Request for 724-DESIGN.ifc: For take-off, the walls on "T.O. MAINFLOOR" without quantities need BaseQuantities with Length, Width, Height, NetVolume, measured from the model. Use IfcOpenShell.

First a look at what the model holds.

```python
import ifcopenshell
import ifcopenshell.util.element
import ifcopenshell.util.unit

model = ifcopenshell.open("724-DESIGN.ifc")
print(model.schema)
for unit_type in ("LENGTHUNIT", "AREAUNIT", "VOLUMEUNIT"):
    print(unit_type, ifcopenshell.util.unit.calculate_unit_scale(model, unit_type))
storey = next(s for s in model.by_type("IfcBuildingStorey") if s.Name == "T.O. MAINFLOOR")
walls = [e for e in ifcopenshell.util.element.get_decomposition(storey) if e.is_a("IfcWall")]
for e in sorted(walls, key=lambda e: e.id()):
    print(e.id(), e.is_a(), e.Name, list(ifcopenshell.util.element.get_psets(e, qtos_only=True)), sep=" | ")
```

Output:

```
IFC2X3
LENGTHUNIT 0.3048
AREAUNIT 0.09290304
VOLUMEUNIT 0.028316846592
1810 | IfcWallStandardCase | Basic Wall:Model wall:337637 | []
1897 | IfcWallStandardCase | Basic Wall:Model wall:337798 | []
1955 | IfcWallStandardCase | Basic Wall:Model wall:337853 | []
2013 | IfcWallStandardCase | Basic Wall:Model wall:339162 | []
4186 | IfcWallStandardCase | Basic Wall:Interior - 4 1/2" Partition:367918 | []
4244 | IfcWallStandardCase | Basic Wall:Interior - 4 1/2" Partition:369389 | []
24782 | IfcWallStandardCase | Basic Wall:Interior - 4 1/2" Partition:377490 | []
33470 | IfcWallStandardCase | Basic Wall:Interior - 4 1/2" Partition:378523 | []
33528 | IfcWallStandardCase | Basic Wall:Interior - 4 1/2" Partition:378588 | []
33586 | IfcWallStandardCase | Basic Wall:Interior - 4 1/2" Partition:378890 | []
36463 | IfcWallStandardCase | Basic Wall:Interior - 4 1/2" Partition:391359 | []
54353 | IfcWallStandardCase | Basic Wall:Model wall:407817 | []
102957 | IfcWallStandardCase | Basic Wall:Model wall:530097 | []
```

```python
import ifcopenshell
import ifcopenshell.api.pset
import ifcopenshell.geom
import ifcopenshell.util.element
import ifcopenshell.util.shape
import ifcopenshell.util.unit

model = ifcopenshell.open("724-DESIGN.ifc")
unit_scale = ifcopenshell.util.unit.calculate_unit_scale(model)
volume_scale = ifcopenshell.util.unit.calculate_unit_scale(model, "VOLUMEUNIT")
settings = ifcopenshell.geom.settings()

storey = next(s for s in model.by_type("IfcBuildingStorey") if s.Name == "T.O. MAINFLOOR")
walls = [e for e in ifcopenshell.util.element.get_decomposition(storey) if e.is_a("IfcWall")]

for e in sorted(walls, key=lambda e: e.id()):
    if ifcopenshell.util.element.get_psets(e, qtos_only=True, should_inherit=False):
        continue
    # Geometry comes back in metres, in the element's own axes.
    shape = ifcopenshell.geom.create_shape(settings, e)
    values = {
        "Length": ifcopenshell.util.shape.get_x(shape.geometry) / unit_scale,
        "Width": ifcopenshell.util.shape.get_y(shape.geometry) / unit_scale,
        "Height": ifcopenshell.util.shape.get_z(shape.geometry) / unit_scale,
        "NetVolume": ifcopenshell.util.shape.get_volume(shape.geometry) / volume_scale,
    }
    qto = ifcopenshell.api.pset.add_qto(model, product=e, name="BaseQuantities")
    ifcopenshell.api.pset.edit_qto(model, qto=qto, properties=values)
    print(e.id(), {k: round(v, 3) for k, v in values.items()})

model.write("724-DESIGN_updated.ifc")
```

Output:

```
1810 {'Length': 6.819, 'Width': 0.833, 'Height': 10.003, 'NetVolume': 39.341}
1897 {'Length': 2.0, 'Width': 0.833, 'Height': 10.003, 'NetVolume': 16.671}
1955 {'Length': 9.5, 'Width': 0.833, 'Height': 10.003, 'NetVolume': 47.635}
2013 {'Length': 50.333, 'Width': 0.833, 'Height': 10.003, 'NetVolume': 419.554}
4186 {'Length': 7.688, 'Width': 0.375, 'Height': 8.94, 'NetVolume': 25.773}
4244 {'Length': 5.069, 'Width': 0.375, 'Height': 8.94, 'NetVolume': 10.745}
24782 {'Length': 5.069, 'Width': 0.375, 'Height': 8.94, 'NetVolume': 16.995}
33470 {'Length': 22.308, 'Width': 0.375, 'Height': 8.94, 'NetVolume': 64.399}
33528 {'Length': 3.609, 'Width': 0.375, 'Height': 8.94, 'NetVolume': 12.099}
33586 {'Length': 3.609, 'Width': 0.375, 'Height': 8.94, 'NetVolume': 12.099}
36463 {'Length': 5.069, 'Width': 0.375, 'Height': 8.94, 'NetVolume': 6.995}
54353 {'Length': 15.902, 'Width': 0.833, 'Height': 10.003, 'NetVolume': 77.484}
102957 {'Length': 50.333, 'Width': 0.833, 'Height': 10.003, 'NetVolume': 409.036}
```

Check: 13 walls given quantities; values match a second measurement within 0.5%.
